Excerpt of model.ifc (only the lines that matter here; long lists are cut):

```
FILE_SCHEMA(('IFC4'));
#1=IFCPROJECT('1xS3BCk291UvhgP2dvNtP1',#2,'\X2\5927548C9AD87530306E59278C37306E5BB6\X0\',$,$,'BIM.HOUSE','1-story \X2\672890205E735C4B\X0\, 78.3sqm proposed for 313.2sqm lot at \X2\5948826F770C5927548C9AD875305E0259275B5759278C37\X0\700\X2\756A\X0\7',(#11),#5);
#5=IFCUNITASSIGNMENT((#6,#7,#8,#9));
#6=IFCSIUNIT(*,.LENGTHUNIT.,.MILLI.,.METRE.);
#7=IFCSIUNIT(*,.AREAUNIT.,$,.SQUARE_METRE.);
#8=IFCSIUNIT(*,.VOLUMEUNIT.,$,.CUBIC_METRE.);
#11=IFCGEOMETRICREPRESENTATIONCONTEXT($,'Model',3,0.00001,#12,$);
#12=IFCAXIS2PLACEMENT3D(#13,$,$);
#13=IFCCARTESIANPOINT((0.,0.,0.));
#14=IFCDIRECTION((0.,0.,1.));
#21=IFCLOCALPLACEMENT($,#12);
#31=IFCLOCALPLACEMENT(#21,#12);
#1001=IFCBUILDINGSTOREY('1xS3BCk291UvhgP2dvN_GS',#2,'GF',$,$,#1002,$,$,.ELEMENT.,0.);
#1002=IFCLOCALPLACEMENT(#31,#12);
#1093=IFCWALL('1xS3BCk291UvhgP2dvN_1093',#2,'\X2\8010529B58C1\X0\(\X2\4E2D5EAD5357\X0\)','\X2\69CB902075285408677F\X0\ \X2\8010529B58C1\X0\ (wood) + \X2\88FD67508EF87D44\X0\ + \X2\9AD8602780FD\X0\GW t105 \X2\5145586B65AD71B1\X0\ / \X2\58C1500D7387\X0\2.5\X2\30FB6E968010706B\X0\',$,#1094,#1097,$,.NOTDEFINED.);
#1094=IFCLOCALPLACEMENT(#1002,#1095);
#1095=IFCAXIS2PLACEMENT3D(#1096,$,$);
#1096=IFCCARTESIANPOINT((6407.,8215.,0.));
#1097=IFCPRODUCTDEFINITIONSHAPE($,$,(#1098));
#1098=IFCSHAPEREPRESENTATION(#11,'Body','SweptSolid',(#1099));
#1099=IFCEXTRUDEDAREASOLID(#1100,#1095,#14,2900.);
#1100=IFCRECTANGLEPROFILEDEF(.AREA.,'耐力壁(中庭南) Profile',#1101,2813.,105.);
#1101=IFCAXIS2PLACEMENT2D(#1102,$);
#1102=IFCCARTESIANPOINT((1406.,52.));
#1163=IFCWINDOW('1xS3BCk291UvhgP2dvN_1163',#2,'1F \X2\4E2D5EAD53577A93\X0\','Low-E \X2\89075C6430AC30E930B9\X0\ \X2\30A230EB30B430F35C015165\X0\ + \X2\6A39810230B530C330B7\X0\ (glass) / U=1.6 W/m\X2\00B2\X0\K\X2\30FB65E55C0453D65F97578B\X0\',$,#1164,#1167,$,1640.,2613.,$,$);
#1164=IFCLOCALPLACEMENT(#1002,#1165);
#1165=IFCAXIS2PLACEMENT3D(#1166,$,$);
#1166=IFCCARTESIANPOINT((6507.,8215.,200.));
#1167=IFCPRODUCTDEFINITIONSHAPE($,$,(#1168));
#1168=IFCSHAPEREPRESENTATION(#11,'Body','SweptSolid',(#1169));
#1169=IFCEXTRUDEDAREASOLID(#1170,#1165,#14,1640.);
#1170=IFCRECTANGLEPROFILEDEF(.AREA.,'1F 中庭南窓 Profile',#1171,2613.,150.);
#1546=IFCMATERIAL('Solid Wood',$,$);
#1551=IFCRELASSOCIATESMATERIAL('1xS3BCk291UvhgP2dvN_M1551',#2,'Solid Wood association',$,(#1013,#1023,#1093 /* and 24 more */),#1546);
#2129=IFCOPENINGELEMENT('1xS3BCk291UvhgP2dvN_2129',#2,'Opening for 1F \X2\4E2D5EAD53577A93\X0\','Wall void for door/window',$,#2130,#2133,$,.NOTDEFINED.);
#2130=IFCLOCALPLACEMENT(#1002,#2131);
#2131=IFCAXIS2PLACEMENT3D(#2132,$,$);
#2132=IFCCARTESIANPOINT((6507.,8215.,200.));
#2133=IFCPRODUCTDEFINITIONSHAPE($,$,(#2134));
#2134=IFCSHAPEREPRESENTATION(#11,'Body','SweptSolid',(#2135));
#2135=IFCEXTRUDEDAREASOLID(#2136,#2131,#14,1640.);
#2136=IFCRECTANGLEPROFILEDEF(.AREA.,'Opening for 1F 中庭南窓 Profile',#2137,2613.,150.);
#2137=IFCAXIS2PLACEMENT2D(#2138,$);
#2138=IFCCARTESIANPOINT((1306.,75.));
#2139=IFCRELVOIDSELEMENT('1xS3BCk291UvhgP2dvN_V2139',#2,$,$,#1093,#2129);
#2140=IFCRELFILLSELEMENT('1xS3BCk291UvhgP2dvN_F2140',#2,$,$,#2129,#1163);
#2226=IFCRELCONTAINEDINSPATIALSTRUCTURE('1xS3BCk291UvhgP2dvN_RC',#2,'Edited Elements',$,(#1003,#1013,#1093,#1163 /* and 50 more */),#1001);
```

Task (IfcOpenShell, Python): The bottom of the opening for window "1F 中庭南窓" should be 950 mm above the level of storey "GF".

```python
import numpy as np
import ifcopenshell
import ifcopenshell.api.geometry
import ifcopenshell.geom
import ifcopenshell.util.element
import ifcopenshell.util.placement
import ifcopenshell.util.shape
import ifcopenshell.util.unit

model = ifcopenshell.open("model.ifc")
unit_scale = ifcopenshell.util.unit.calculate_unit_scale(model)

window = model.by_id(1163)
opening = window.FillsVoids[0].RelatingOpeningElement
storey = ifcopenshell.util.element.get_container(window, ifc_class="IfcBuildingStorey")
level = ifcopenshell.util.placement.get_local_placement(storey.ObjectPlacement)[2, 3]

# The opening's origin need not be at the sill, so measure its lowest point.
shape = ifcopenshell.geom.create_shape(ifcopenshell.geom.settings(), opening)
bottom = ifcopenshell.util.shape.get_shape_bottom_elevation(shape, shape.geometry) / unit_scale
dz = level + 0.95 / unit_scale - bottom

shift = np.array([0.0, 0.0, dz])
# The window is not placed relative to its opening, so move both.
for product in (opening, window):
    matrix = ifcopenshell.util.placement.get_local_placement(product.ObjectPlacement)
    matrix[:3, 3] += shift
    ifcopenshell.api.geometry.edit_object_placement(model, product=product, matrix=matrix, is_si=False)

print(f"moved by {dz * unit_scale:+.3f} m")

model.write("model_edited.ifc")
```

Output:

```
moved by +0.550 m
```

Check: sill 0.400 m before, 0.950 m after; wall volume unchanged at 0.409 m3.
